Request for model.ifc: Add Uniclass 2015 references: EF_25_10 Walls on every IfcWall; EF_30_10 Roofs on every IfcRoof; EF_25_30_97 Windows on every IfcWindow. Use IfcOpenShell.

First a look at what the model holds.

```python
import ifcopenshell

model = ifcopenshell.open("model.ifc")
print(model.schema)
print("classifications:", [c.Name for c in model.by_type("IfcClassification")])
for ifc_class in ("IfcDoor", "IfcRoof", "IfcStair", "IfcWall", "IfcWindow"):
    print(ifc_class, len(model.by_type(ifc_class)))
```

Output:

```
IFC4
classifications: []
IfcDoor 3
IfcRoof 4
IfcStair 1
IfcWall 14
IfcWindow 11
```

```python
import ifcopenshell
import ifcopenshell.api.classification

model = ifcopenshell.open("model.ifc")

system = ifcopenshell.api.classification.add_classification(model, classification="Uniclass 2015")

codes = {
    "IfcWall": ("EF_25_10", "Walls"),
    "IfcRoof": ("EF_30_10", "Roofs"),
    "IfcWindow": ("EF_25_30_97", "Windows"),
}
for ifc_class, (code, name) in codes.items():
    products = model.by_type(ifc_class)
    ifcopenshell.api.classification.add_reference(
        model, products=products, classification=system, identification=code, name=name
    )
    print(code, len(products))

model.write("model_v2.ifc")
```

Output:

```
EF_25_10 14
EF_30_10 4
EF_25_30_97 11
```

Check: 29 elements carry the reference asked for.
